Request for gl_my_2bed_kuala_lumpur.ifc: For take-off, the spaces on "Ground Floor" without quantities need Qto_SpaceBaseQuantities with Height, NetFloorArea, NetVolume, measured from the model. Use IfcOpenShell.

First a look at what the model holds.

```python
import ifcopenshell
import ifcopenshell.util.element
import ifcopenshell.util.unit

model = ifcopenshell.open("gl_my_2bed_kuala_lumpur.ifc")
print(model.schema)
for unit_type in ("LENGTHUNIT", "AREAUNIT", "VOLUMEUNIT"):
    print(unit_type, ifcopenshell.util.unit.calculate_unit_scale(model, unit_type))
storey = next(s for s in model.by_type("IfcBuildingStorey") if s.Name == "Ground Floor")
spaces = [e for e in ifcopenshell.util.element.get_decomposition(storey) if e.is_a("IfcSpace")]
for e in sorted(spaces, key=lambda e: e.id()):
    print(e.id(), e.is_a(), e.Name, list(ifcopenshell.util.element.get_psets(e, qtos_only=True)), sep=" | ")
```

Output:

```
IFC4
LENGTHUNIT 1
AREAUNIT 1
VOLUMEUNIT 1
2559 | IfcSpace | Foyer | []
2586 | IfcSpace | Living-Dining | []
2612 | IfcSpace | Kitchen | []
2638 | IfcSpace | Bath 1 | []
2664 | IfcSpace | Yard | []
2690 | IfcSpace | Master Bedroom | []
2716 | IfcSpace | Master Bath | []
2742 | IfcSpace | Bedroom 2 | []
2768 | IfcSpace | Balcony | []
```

```python
import ifcopenshell
import ifcopenshell.api.pset
import ifcopenshell.geom
import ifcopenshell.util.element
import ifcopenshell.util.shape
import ifcopenshell.util.unit

model = ifcopenshell.open("gl_my_2bed_kuala_lumpur.ifc")
unit_scale = ifcopenshell.util.unit.calculate_unit_scale(model)
area_scale = ifcopenshell.util.unit.calculate_unit_scale(model, "AREAUNIT")
volume_scale = ifcopenshell.util.unit.calculate_unit_scale(model, "VOLUMEUNIT")
settings = ifcopenshell.geom.settings()

storey = next(s for s in model.by_type("IfcBuildingStorey") if s.Name == "Ground Floor")
spaces = [e for e in ifcopenshell.util.element.get_decomposition(storey) if e.is_a("IfcSpace")]

for e in sorted(spaces, key=lambda e: e.id()):
    if ifcopenshell.util.element.get_psets(e, qtos_only=True, should_inherit=False):
        continue
    # Geometry comes back in metres, in the element's own axes.
    shape = ifcopenshell.geom.create_shape(settings, e)
    values = {
        "Height": ifcopenshell.util.shape.get_z(shape.geometry) / unit_scale,
        "NetFloorArea": ifcopenshell.util.shape.get_footprint_area(shape.geometry) / area_scale,
        "NetVolume": ifcopenshell.util.shape.get_volume(shape.geometry) / volume_scale,
    }
    qto = ifcopenshell.api.pset.add_qto(model, product=e, name="Qto_SpaceBaseQuantities")
    ifcopenshell.api.pset.edit_qto(model, qto=qto, properties=values)
    print(e.id(), {k: round(v, 3) for k, v in values.items()})

model.write("gl_my_2bed_kuala_lumpur_updated.ifc")
```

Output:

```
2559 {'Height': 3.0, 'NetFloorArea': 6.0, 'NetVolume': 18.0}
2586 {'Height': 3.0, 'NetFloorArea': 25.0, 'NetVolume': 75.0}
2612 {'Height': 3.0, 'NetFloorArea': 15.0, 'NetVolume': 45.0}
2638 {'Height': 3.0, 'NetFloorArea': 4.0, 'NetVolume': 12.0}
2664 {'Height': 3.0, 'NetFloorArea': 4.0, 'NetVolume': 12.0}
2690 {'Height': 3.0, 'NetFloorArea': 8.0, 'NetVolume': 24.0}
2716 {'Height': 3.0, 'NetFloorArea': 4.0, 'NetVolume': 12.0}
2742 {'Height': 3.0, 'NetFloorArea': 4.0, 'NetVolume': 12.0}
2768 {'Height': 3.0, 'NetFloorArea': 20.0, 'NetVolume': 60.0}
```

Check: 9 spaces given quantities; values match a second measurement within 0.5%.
